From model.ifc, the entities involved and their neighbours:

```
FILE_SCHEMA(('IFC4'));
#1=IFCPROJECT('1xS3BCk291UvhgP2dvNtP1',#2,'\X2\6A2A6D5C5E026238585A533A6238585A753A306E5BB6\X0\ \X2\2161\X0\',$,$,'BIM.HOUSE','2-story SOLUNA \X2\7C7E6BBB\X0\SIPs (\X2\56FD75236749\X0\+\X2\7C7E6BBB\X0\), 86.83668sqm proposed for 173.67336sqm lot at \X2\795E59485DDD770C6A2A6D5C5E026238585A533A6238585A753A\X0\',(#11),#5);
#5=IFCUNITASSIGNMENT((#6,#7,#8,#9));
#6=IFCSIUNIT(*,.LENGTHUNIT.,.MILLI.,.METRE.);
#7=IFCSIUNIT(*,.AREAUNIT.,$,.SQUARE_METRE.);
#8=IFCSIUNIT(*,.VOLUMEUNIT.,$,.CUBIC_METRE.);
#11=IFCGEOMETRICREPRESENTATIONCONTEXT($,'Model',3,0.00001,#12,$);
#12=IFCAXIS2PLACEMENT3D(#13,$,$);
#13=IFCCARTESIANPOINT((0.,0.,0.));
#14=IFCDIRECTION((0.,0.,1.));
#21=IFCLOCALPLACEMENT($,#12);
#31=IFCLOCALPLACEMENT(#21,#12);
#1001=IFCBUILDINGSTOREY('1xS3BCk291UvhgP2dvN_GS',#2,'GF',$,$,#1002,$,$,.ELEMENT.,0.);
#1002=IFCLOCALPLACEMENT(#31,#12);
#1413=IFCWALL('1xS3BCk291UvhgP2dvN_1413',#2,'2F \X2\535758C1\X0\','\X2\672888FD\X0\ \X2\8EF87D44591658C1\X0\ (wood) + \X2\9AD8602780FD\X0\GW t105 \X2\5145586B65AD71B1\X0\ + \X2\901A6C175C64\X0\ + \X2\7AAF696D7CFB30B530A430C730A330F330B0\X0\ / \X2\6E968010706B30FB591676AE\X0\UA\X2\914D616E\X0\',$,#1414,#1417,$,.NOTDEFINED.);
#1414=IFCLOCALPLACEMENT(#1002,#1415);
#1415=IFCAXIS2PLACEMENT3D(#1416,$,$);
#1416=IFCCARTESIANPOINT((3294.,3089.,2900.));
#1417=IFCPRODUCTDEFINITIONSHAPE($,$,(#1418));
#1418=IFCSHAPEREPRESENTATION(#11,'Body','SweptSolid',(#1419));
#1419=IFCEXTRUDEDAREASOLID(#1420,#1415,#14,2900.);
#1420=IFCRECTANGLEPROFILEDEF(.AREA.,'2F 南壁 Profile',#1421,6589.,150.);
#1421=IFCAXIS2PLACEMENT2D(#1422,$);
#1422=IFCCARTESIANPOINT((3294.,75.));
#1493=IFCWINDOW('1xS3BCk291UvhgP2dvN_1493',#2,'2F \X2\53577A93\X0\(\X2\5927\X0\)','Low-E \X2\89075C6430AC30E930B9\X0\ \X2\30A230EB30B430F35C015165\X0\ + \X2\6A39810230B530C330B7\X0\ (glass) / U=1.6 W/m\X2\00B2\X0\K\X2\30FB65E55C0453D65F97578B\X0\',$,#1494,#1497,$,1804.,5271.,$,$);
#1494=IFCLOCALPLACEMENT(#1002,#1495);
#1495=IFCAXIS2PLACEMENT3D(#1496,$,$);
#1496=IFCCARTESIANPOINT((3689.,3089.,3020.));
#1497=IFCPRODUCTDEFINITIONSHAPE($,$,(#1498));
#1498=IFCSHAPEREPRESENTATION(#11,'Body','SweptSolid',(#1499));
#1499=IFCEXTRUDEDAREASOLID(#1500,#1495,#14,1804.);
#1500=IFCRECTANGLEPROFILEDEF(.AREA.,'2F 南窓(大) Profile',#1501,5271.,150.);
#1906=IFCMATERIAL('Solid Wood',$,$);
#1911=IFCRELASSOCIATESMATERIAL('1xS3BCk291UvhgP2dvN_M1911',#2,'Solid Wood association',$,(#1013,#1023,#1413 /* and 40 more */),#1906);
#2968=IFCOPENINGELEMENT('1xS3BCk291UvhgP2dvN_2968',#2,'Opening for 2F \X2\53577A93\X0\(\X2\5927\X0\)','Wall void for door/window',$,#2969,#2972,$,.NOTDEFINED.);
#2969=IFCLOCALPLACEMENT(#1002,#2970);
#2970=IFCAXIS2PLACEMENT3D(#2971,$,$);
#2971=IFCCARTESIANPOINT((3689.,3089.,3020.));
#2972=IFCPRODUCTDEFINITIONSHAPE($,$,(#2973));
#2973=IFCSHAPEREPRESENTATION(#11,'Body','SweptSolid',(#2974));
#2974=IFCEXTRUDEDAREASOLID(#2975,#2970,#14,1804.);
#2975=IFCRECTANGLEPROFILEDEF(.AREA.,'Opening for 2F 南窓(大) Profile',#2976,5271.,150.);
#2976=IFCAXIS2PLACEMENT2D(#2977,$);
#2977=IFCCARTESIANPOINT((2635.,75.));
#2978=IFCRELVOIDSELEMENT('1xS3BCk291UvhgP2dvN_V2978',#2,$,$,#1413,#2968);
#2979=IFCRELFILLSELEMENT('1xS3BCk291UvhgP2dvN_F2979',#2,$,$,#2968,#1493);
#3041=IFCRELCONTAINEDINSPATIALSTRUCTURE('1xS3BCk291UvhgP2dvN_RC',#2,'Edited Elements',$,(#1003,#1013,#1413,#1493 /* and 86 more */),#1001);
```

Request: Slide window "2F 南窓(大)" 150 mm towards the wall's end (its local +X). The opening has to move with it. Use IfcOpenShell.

```python
import ifcopenshell
import ifcopenshell.api.geometry
import ifcopenshell.util.placement
import ifcopenshell.util.unit

model = ifcopenshell.open("model.ifc")
unit_scale = ifcopenshell.util.unit.calculate_unit_scale(model)

window = model.by_guid("1xS3BCk291UvhgP2dvN_1493")
opening = window.FillsVoids[0].RelatingOpeningElement
wall = opening.VoidsElements[0].RelatingBuildingElement

wall_matrix = ifcopenshell.util.placement.get_local_placement(wall.ObjectPlacement)
shift = wall_matrix[:3, 0] * 0.15 / unit_scale
before = ifcopenshell.util.placement.get_local_placement(window.ObjectPlacement)[:3, 3].copy()

# The window is not placed relative to its opening, so move both.
for product in (opening, window):
    matrix = ifcopenshell.util.placement.get_local_placement(product.ObjectPlacement)
    matrix[:3, 3] += shift
    ifcopenshell.api.geometry.edit_object_placement(model, product=product, matrix=matrix, is_si=False)

after = ifcopenshell.util.placement.get_local_placement(window.ObjectPlacement)[:3, 3]
print("window moved by", (after - before).round(3) + 0.0)

model.write("model_updated.ifc")
```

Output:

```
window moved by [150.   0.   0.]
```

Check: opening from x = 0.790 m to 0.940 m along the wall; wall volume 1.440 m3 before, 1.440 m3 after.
